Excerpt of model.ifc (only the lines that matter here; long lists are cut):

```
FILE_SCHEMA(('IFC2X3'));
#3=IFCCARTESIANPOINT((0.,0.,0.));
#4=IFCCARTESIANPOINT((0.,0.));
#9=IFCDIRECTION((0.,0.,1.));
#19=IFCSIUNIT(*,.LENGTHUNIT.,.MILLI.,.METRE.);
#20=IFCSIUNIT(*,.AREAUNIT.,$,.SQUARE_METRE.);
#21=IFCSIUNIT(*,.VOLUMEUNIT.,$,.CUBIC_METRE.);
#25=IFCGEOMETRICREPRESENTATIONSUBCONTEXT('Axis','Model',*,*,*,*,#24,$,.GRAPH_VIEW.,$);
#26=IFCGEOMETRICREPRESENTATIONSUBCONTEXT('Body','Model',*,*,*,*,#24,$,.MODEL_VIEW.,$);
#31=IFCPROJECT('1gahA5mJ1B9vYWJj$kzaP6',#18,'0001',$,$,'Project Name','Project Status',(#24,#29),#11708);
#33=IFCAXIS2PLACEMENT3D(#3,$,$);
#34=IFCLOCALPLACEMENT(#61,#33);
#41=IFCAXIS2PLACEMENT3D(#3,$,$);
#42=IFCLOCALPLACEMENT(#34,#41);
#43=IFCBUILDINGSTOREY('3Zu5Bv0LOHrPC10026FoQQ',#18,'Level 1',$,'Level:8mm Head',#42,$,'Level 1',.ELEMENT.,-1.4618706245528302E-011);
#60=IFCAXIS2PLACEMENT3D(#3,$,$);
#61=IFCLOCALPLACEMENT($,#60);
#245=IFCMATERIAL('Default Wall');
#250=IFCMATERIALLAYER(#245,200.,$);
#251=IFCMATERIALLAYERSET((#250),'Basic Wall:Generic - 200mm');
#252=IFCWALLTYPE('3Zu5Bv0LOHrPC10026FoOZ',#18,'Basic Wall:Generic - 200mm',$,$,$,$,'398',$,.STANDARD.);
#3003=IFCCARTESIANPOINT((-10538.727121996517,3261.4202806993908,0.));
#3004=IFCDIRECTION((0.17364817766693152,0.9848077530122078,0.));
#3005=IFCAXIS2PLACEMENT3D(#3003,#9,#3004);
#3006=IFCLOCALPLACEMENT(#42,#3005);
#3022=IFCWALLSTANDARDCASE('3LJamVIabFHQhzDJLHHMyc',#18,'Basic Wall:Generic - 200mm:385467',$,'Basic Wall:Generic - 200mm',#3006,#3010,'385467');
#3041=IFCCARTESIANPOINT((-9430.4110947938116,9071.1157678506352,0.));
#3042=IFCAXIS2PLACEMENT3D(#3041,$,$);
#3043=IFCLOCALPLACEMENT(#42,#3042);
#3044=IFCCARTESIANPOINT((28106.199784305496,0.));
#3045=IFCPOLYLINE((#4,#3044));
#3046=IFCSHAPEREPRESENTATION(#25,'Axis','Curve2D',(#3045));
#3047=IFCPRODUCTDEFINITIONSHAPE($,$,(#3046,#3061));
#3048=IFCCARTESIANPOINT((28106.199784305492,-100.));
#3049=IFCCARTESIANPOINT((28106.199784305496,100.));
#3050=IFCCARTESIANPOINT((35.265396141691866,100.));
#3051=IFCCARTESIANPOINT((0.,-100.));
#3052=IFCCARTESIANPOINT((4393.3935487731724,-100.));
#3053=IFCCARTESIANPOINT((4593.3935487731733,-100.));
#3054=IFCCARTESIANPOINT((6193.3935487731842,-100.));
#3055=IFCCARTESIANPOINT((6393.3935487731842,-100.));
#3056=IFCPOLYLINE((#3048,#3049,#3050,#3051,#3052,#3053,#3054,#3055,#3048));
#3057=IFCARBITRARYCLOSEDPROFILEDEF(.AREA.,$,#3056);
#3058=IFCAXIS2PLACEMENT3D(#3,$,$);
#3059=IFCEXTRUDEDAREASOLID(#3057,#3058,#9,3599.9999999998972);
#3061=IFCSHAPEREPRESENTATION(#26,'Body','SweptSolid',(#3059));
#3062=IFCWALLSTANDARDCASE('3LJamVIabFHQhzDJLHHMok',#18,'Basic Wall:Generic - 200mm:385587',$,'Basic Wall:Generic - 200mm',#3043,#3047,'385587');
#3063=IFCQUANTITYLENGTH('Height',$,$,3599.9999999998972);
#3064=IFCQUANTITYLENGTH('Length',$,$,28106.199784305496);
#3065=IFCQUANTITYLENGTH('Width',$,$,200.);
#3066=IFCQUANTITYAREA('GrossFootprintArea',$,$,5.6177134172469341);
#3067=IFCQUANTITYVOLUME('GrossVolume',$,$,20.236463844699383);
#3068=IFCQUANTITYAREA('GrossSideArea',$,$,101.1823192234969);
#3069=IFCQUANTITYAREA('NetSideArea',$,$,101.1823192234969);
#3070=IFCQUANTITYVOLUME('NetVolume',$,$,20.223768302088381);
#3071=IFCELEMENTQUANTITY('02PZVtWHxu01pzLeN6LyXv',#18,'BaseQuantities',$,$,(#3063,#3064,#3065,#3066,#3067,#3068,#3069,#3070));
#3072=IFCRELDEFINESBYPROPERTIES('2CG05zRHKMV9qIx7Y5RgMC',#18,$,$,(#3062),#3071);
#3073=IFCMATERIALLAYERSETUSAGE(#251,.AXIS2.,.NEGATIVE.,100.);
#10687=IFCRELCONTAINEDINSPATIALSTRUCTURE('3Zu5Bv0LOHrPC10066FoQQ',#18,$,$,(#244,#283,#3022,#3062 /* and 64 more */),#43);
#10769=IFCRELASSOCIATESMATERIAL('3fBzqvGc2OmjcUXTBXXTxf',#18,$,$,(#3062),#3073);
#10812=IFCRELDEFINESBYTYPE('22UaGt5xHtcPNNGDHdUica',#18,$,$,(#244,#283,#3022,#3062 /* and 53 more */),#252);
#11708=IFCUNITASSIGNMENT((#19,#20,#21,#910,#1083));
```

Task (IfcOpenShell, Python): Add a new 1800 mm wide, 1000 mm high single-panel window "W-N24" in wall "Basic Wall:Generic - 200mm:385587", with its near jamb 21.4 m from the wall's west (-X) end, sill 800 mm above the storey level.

```python
import numpy as np
import ifcopenshell
import ifcopenshell.api.feature
import ifcopenshell.api.geometry
import ifcopenshell.api.pset
import ifcopenshell.api.root
import ifcopenshell.api.spatial
import ifcopenshell.api.type
import ifcopenshell.geom
import ifcopenshell.util.element
import ifcopenshell.util.placement
import ifcopenshell.util.representation
import ifcopenshell.util.shape
import ifcopenshell.util.unit

model = ifcopenshell.open("model.ifc")
unit_scale = ifcopenshell.util.unit.calculate_unit_scale(model)
area_scale = ifcopenshell.util.unit.calculate_unit_scale(model, "AREAUNIT")
volume_scale = ifcopenshell.util.unit.calculate_unit_scale(model, "VOLUMEUNIT")
settings = ifcopenshell.geom.settings()


def volume(element):
    """Net volume in cubic metres, openings subtracted."""
    shape = ifcopenshell.geom.create_shape(settings, element)
    return ifcopenshell.util.shape.get_volume(shape.geometry)


wall = model.by_guid("3LJamVIabFHQhzDJLHHMok")
storey = ifcopenshell.util.element.get_container(wall, ifc_class="IfcBuildingStorey")
context = ifcopenshell.util.representation.get_context(model, "Model", "Body", "MODEL_VIEW")
before = volume(wall)

width, height, from_end, sill = 1.8, 1, 21.4, 0.8  # metres

# The wall runs along its own X axis, and the end named is its -X end.
wall_shape = ifcopenshell.geom.create_shape(settings, wall)
x, y, z = ifcopenshell.util.shape.get_vertices(wall_shape.geometry).T
start = x.min() + from_end
face, thickness = float(y.min()), float(y.max() - y.min())
wall_matrix = ifcopenshell.util.placement.get_local_placement(wall.ObjectPlacement)
level = ifcopenshell.util.placement.get_local_placement(storey.ObjectPlacement)[2, 3]


def in_wall(x, y):
    """Placement at x, y metres in the wall's axes, at sill height."""
    matrix = wall_matrix.copy()
    matrix[:, 3] = wall_matrix @ np.array([x / unit_scale, y / unit_scale, 0.0, 1.0])
    matrix[2, 3] = level + sill / unit_scale
    return matrix


# Opening: a box that overshoots both wall faces by 50 mm.
opening = ifcopenshell.api.root.create_entity(model, ifc_class="IfcOpeningElement")
box = ifcopenshell.api.geometry.add_wall_representation(
    model, context=context, length=width, height=height, thickness=thickness + 0.1
)
ifcopenshell.api.geometry.assign_representation(model, product=opening, representation=box)
ifcopenshell.api.geometry.edit_object_placement(model, product=opening, matrix=in_wall(start, face - 0.05), is_si=False)
ifcopenshell.api.feature.add_feature(model, feature=opening, element=wall)

window = ifcopenshell.api.root.create_entity(model, ifc_class="IfcWindow", name="W-N24")
window.OverallWidth, window.OverallHeight = width / unit_scale, height / unit_scale
body = ifcopenshell.api.geometry.add_window_representation(
    model,
    context=context,
    overall_width=window.OverallWidth,
    overall_height=window.OverallHeight,
    partition_type="SINGLE_PANEL",
)
ifcopenshell.api.geometry.assign_representation(model, product=window, representation=body)
ifcopenshell.api.spatial.assign_container(model, products=[window], relating_structure=storey)
fills = ifcopenshell.api.feature.add_filling(model, opening=opening, element=window)
fills.OwnerHistory = window.OwnerHistory  # required in IFC2X3

# IFC2X3 keeps the operation on the window style.
style = ifcopenshell.api.root.create_entity(model, ifc_class="IfcWindowStyle", name="W-N24")
style.OperationType, style.ConstructionType = "SINGLE_PANEL", "NOTDEFINED"
style.ParameterTakesPrecedence = style.Sizeable = False
ifcopenshell.api.type.assign_type(model, related_objects=[window], relating_type=style)

# Centre the window in the wall's thickness.
ifcopenshell.api.geometry.edit_object_placement(model, product=window, matrix=in_wall(start, face), is_si=False)
window_shape = ifcopenshell.geom.create_shape(settings, window)
depth = ifcopenshell.util.shape.get_vertices(window_shape.geometry)[:, 1]
offset = face + thickness / 2 - (depth.min() + depth.max()) / 2
ifcopenshell.api.geometry.edit_object_placement(model, product=window, matrix=in_wall(start, offset), is_si=False)

after = volume(wall)

# Update the wall's stored quantities.
qto = model.by_id(ifcopenshell.util.element.get_pset(wall, "BaseQuantities", should_inherit=False)["id"])
ifcopenshell.api.pset.edit_qto(model, qto=qto, properties={
    "NetSideArea": after / thickness / area_scale,
    "NetVolume": after / volume_scale,
})

print(f"wall volume {before:.3f} -> {after:.3f} m3")

model.write("model_updated.ifc")
```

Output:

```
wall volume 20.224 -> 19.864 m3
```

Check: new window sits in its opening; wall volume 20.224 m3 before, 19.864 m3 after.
